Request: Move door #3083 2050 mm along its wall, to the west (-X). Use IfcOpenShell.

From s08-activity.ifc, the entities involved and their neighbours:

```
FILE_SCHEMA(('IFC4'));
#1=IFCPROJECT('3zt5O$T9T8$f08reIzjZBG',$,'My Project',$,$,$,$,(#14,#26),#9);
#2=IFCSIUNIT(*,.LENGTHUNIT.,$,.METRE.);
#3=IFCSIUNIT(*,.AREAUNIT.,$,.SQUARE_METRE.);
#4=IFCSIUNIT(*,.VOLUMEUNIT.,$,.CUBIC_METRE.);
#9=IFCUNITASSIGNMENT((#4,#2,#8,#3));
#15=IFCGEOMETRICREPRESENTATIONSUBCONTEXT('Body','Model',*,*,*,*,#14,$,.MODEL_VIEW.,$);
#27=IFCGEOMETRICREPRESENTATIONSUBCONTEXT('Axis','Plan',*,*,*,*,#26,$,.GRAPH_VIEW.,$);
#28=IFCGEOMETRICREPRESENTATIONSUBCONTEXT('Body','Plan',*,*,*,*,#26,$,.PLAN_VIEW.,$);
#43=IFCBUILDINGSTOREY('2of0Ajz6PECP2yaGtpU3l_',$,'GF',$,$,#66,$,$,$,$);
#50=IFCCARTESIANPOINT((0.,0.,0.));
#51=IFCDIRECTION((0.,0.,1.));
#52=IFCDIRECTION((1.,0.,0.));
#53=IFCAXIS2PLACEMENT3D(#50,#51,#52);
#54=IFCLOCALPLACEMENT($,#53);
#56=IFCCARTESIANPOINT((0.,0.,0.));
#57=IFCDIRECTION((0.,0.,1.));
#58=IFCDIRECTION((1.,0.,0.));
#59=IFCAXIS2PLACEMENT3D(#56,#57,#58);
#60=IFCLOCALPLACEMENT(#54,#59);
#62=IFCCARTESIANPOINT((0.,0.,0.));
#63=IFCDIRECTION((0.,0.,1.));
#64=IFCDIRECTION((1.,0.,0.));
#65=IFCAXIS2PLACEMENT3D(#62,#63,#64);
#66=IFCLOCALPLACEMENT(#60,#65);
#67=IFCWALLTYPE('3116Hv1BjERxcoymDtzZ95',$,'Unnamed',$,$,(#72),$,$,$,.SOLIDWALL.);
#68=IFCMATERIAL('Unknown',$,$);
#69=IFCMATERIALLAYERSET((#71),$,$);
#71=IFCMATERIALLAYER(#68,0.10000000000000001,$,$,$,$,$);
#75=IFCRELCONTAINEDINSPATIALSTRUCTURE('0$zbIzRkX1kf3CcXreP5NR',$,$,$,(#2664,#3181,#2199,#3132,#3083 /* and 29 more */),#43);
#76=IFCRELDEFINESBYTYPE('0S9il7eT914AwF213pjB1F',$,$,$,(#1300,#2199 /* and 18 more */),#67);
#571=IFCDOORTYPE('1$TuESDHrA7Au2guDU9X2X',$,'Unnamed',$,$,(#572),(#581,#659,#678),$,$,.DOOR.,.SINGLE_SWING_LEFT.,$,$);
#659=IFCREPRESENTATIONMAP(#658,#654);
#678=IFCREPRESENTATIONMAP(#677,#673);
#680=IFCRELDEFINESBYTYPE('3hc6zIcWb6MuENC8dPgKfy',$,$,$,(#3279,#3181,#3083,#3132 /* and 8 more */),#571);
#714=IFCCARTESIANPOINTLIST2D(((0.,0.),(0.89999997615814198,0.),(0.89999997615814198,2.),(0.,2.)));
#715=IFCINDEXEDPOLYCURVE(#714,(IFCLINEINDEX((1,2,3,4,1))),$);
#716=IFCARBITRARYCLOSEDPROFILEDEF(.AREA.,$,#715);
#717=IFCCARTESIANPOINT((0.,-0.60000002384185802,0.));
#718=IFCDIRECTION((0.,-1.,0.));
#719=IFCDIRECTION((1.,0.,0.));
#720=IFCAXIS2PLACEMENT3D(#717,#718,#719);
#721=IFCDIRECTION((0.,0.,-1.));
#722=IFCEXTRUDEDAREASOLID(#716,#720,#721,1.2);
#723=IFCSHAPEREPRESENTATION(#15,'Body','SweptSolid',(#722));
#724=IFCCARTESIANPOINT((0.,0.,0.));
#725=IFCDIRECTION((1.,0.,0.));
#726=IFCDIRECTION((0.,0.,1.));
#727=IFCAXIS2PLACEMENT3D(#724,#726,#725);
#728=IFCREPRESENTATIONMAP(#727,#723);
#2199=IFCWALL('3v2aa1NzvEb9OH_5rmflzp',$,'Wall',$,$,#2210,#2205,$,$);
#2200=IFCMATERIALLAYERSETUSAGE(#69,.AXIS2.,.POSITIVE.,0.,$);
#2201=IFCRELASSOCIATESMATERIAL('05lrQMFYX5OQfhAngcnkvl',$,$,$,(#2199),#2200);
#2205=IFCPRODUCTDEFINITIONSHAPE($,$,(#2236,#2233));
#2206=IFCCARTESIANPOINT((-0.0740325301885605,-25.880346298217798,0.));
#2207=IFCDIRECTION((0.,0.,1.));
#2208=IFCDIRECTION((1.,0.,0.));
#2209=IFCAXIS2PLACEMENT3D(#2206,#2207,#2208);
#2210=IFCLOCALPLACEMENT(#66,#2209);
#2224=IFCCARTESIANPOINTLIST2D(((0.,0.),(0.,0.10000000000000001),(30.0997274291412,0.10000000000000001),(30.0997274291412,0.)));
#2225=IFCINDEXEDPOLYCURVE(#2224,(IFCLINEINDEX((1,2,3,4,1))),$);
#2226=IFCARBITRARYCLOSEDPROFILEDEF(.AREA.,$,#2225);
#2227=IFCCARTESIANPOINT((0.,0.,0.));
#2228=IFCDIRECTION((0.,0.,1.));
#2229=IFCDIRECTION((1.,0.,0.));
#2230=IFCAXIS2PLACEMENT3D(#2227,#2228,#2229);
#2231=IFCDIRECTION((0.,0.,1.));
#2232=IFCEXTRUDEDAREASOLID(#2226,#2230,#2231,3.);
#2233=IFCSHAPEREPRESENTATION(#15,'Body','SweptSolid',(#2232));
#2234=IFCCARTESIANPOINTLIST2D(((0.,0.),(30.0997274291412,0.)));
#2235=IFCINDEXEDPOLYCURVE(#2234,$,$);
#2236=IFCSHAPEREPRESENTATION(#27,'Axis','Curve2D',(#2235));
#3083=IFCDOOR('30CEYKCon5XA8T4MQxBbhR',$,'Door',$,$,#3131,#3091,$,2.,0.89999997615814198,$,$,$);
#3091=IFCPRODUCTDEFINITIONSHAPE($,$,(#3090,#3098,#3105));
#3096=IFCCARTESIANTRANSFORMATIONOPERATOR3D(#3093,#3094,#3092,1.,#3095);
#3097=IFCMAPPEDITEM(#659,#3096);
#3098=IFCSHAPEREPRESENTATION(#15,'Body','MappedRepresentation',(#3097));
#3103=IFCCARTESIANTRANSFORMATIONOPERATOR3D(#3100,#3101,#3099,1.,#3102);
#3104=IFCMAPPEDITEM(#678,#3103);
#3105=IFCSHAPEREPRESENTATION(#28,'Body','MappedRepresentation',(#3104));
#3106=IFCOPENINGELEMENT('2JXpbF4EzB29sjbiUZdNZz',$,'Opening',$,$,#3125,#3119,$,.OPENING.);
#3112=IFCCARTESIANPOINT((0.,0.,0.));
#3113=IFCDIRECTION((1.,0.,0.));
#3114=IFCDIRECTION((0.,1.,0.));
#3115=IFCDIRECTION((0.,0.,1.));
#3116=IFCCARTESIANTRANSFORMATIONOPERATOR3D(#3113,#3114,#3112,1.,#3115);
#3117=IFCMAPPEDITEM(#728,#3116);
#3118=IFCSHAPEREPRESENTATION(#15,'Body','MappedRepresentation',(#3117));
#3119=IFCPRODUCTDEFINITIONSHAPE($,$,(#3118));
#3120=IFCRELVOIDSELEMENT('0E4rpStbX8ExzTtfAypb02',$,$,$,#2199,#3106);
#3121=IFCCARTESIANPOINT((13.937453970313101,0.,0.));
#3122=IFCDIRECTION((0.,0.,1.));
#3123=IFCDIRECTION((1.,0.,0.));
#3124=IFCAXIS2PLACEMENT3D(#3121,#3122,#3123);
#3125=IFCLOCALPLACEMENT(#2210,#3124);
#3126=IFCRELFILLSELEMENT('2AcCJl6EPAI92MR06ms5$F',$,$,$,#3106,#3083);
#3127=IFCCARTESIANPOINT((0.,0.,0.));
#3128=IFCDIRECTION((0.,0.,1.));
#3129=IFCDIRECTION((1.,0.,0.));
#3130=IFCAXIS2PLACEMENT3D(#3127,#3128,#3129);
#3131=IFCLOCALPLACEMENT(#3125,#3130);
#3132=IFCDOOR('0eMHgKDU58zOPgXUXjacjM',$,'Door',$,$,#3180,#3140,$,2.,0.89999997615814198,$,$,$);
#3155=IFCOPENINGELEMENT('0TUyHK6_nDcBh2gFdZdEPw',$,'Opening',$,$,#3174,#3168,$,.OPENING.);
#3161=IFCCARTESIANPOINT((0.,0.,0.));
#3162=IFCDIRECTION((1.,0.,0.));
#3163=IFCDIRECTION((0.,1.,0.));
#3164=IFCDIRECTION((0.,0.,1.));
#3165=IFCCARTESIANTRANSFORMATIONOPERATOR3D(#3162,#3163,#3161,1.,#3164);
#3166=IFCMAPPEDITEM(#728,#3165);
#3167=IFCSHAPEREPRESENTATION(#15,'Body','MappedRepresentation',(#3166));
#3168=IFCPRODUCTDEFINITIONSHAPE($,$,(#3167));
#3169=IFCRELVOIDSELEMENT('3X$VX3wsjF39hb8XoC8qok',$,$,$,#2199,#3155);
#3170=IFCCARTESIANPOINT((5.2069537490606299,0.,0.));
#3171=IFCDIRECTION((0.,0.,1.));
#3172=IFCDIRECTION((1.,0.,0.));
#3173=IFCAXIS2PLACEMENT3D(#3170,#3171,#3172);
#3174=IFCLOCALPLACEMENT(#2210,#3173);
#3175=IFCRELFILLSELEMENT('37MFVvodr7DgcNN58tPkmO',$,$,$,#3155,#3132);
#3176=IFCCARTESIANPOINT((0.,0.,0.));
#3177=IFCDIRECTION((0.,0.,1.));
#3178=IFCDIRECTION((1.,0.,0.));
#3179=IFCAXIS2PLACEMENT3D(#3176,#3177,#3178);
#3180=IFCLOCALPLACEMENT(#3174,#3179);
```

```python
import ifcopenshell
import ifcopenshell.api.geometry
import ifcopenshell.util.placement
import ifcopenshell.util.unit

model = ifcopenshell.open("s08-activity.ifc")
unit_scale = ifcopenshell.util.unit.calculate_unit_scale(model)

door = model.by_guid("30CEYKCon5XA8T4MQxBbhR")
opening = door.FillsVoids[0].RelatingOpeningElement
wall = opening.VoidsElements[0].RelatingBuildingElement

wall_matrix = ifcopenshell.util.placement.get_local_placement(wall.ObjectPlacement)
shift = wall_matrix[:3, 0] * -2.05 / unit_scale
before = ifcopenshell.util.placement.get_local_placement(door.ObjectPlacement)[:3, 3].copy()

# The door is placed relative to its opening, so it follows when the opening moves.
matrix = ifcopenshell.util.placement.get_local_placement(opening.ObjectPlacement)
matrix[:3, 3] += shift
ifcopenshell.api.geometry.edit_object_placement(
    model, product=opening, matrix=matrix, is_si=False, should_transform_children=True
)

after = ifcopenshell.util.placement.get_local_placement(door.ObjectPlacement)[:3, 3]
print("door moved by", (after - before).round(3) + 0.0)

model.write("s08-activity_edited.ifc")
```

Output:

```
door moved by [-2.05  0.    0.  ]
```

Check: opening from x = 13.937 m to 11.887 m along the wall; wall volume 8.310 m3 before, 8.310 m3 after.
